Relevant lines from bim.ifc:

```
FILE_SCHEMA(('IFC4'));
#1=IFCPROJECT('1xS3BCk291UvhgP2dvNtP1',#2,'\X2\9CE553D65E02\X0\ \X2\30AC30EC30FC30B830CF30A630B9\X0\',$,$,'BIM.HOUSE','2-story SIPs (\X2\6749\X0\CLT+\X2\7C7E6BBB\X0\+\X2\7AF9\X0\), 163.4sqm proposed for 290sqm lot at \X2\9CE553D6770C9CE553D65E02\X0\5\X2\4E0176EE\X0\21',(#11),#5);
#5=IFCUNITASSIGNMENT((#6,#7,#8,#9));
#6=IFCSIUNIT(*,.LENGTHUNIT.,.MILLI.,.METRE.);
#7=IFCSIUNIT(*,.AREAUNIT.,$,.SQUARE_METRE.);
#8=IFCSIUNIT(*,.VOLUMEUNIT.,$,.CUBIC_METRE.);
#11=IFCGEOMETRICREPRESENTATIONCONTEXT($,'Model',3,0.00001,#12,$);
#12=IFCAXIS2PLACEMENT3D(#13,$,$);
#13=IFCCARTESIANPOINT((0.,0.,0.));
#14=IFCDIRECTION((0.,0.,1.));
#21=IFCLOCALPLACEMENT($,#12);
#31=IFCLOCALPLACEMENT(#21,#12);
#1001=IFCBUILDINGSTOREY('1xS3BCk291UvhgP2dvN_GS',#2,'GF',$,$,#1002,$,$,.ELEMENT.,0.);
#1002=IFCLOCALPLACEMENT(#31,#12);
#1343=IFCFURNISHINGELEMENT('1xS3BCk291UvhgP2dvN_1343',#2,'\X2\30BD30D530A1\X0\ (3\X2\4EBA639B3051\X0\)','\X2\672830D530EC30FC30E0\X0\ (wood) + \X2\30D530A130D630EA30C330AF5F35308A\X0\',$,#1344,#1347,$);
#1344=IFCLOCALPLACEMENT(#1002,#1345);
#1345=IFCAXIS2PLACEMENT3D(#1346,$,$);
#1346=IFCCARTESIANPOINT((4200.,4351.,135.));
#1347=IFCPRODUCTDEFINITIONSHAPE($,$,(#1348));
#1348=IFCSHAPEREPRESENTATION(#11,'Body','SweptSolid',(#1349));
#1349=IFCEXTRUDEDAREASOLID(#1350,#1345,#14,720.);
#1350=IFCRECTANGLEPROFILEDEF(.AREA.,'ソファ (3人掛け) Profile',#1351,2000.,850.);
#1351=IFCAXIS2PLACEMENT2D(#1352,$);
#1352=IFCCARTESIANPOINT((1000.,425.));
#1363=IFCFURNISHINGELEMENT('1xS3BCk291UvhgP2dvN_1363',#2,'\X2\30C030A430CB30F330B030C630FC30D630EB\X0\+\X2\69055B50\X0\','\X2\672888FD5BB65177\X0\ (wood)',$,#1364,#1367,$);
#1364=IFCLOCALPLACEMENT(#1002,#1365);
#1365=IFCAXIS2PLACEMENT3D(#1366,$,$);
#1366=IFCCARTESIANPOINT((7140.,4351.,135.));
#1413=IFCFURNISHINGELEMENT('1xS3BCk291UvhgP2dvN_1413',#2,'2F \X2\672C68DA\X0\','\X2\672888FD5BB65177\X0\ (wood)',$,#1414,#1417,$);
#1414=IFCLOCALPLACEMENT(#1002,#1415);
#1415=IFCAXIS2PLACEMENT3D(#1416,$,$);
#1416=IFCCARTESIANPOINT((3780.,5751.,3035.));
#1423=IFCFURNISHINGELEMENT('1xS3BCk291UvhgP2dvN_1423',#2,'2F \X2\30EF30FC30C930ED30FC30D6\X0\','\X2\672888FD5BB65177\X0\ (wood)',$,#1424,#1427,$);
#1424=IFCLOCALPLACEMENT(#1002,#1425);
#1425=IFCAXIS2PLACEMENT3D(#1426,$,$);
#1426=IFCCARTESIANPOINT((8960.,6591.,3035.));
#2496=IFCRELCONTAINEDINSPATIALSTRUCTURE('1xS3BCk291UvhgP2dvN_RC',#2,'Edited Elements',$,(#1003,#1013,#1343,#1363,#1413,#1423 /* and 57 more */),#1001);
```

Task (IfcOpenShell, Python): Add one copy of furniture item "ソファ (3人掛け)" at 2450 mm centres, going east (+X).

```python
import numpy as np
import ifcopenshell
import ifcopenshell.api.geometry
import ifcopenshell.api.root
import ifcopenshell.util.element
import ifcopenshell.util.placement

model = ifcopenshell.open("bim.ifc")


def reuse_history(source, copy):
    """copy_class also copies each property set's owner history, people and application; keep the originals."""
    for rel in copy.IsDefinedBy:
        if rel.is_a("IfcRelDefinesByProperties") and (history := rel.RelatingPropertyDefinition.OwnerHistory):
            rel.RelatingPropertyDefinition.OwnerHistory = source.OwnerHistory
            ifcopenshell.util.element.remove_deep2(model, history)


source = model.by_guid("1xS3BCk291UvhgP2dvN_1343")
base = ifcopenshell.util.placement.get_local_placement(source.ObjectPlacement)
step = np.array([1.0, 0.0, 0.0]) * 2450.0

for i in range(1, 2):
    copy = ifcopenshell.api.root.copy_class(model, product=source)
    copy.Representation = ifcopenshell.util.element.copy_deep(
        model, source.Representation, exclude=["IfcGeometricRepresentationContext", "IfcRepresentationMap"]
    )
    reuse_history(source, copy)
    matrix = base.copy()
    matrix[:3, 3] += i * step
    print("added at", matrix[:3, 3].round(3) + 0.0)
    ifcopenshell.api.geometry.edit_object_placement(model, product=copy, matrix=matrix, is_si=False)

model.write("bim-out.ifc")
```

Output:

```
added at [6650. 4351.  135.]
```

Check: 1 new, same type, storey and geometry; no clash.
